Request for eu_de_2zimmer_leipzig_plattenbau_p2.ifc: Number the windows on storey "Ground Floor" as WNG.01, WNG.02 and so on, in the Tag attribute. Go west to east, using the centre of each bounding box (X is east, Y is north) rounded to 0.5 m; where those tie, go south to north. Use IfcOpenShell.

First a look at what the model holds.

```python
import ifcopenshell
import ifcopenshell.util.element
import ifcopenshell.util.placement

model = ifcopenshell.open("eu_de_2zimmer_leipzig_plattenbau_p2.ifc")
print(model.schema)
storey = next(s for s in model.by_type("IfcBuildingStorey") if s.Name == "Ground Floor")
windows = [e for e in ifcopenshell.util.element.get_decomposition(storey) if e.is_a("IfcWindow")]
for e in sorted(windows, key=lambda e: e.id()):
    origin = ifcopenshell.util.placement.get_local_placement(e.ObjectPlacement)[:3, 3]
    print(e.id(), e.Tag, e.Name, origin.round(2) + 0.0, sep=" | ")
```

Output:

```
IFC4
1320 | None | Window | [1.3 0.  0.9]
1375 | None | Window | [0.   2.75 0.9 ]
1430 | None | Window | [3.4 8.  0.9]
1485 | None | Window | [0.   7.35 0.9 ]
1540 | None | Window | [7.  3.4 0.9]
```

```python
import ifcopenshell
import ifcopenshell.geom
import ifcopenshell.util.element
import ifcopenshell.util.shape

model = ifcopenshell.open("eu_de_2zimmer_leipzig_plattenbau_p2.ifc")
settings = ifcopenshell.geom.settings()
settings.set("use-world-coords", True)


def centre(element):
    shape = ifcopenshell.geom.create_shape(settings, element)
    return ifcopenshell.util.shape.get_bbox_centroid(shape.geometry)


storey = next(s for s in model.by_type("IfcBuildingStorey") if s.Name == "Ground Floor")
windows = [e for e in ifcopenshell.util.element.get_decomposition(storey) if e.is_a("IfcWindow")]

# Insertion points can sit at a corner or the storey origin, so sort by the geometry (in metres).
centres = {e: centre(e) for e in windows}
windows.sort(key=lambda e: (round(centres[e][0] / 0.5), centres[e][1]))

for i, e in enumerate(windows, start=1):
    number = f"WNG.{i:02d}"
    e.Tag = number
    print(e.id(), number)

model.write("eu_de_2zimmer_leipzig_plattenbau_p2_edited.ifc")
```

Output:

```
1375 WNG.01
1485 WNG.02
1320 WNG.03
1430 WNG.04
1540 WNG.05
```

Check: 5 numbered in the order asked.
